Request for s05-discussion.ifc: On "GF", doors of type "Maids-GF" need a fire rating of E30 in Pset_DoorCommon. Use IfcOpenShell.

First a look at what the model holds.

```python
import ifcopenshell
import ifcopenshell.util.element

model = ifcopenshell.open("s05-discussion.ifc")
print(model.schema)
storey = next(s for s in model.by_type("IfcBuildingStorey") if s.Name == "GF")
doors = [e for e in ifcopenshell.util.element.get_decomposition(storey) if e.is_a("IfcDoor")]
seen = {}
for e in doors:
    element_type = ifcopenshell.util.element.get_type(e)
    key = (element_type.Name if element_type != e and element_type else None, ifcopenshell.util.element.get_pset(e, "Pset_DoorCommon", "FireRating"))
    seen[key] = seen.get(key, 0) + 1
for (name, value), count in sorted(seen.items(), key=str):
    print(count, "x", name, "|", value)
```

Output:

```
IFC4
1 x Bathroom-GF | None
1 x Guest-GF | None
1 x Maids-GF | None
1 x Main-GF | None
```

```python
import ifcopenshell
import ifcopenshell.api.pset
import ifcopenshell.util.element

model = ifcopenshell.open("s05-discussion.ifc")

storey = next(s for s in model.by_type("IfcBuildingStorey") if s.Name == "GF")
doors = [e for e in ifcopenshell.util.element.get_decomposition(storey) if e.is_a("IfcDoor")]

count = 0
for e in doors:
    element_type = ifcopenshell.util.element.get_type(e)
    if element_type in (None, e) or element_type.Name != "Maids-GF":
        continue
    # add_pset returns the element's existing set when there is one.
    pset = ifcopenshell.api.pset.add_pset(model, product=e, name="Pset_DoorCommon")
    ifcopenshell.api.pset.edit_pset(model, pset=pset, properties={"FireRating": "E30"})
    count += 1

print(count, "doors updated")

model.write("s05-discussion_v2.ifc")
```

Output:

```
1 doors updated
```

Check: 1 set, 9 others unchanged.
